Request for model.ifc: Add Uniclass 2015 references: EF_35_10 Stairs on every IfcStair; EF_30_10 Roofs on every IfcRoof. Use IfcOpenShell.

First a look at what the model holds.

```python
import ifcopenshell

model = ifcopenshell.open("model.ifc")
print(model.schema)
print("classifications:", [c.Name for c in model.by_type("IfcClassification")])
for ifc_class in ("IfcDoor", "IfcRoof", "IfcStair", "IfcWall", "IfcWindow"):
    print(ifc_class, len(model.by_type(ifc_class)))
```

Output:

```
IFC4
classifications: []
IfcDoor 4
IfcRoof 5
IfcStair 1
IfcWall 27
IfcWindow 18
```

```python
import ifcopenshell
import ifcopenshell.api.classification

model = ifcopenshell.open("model.ifc")

system = ifcopenshell.api.classification.add_classification(model, classification="Uniclass 2015")

codes = {
    "IfcStair": ("EF_35_10", "Stairs"),
    "IfcRoof": ("EF_30_10", "Roofs"),
}
for ifc_class, (code, name) in codes.items():
    products = model.by_type(ifc_class)
    ifcopenshell.api.classification.add_reference(
        model, products=products, classification=system, identification=code, name=name
    )
    print(code, len(products))

model.write("model_v2.ifc")
```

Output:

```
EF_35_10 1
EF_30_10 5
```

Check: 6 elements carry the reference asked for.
